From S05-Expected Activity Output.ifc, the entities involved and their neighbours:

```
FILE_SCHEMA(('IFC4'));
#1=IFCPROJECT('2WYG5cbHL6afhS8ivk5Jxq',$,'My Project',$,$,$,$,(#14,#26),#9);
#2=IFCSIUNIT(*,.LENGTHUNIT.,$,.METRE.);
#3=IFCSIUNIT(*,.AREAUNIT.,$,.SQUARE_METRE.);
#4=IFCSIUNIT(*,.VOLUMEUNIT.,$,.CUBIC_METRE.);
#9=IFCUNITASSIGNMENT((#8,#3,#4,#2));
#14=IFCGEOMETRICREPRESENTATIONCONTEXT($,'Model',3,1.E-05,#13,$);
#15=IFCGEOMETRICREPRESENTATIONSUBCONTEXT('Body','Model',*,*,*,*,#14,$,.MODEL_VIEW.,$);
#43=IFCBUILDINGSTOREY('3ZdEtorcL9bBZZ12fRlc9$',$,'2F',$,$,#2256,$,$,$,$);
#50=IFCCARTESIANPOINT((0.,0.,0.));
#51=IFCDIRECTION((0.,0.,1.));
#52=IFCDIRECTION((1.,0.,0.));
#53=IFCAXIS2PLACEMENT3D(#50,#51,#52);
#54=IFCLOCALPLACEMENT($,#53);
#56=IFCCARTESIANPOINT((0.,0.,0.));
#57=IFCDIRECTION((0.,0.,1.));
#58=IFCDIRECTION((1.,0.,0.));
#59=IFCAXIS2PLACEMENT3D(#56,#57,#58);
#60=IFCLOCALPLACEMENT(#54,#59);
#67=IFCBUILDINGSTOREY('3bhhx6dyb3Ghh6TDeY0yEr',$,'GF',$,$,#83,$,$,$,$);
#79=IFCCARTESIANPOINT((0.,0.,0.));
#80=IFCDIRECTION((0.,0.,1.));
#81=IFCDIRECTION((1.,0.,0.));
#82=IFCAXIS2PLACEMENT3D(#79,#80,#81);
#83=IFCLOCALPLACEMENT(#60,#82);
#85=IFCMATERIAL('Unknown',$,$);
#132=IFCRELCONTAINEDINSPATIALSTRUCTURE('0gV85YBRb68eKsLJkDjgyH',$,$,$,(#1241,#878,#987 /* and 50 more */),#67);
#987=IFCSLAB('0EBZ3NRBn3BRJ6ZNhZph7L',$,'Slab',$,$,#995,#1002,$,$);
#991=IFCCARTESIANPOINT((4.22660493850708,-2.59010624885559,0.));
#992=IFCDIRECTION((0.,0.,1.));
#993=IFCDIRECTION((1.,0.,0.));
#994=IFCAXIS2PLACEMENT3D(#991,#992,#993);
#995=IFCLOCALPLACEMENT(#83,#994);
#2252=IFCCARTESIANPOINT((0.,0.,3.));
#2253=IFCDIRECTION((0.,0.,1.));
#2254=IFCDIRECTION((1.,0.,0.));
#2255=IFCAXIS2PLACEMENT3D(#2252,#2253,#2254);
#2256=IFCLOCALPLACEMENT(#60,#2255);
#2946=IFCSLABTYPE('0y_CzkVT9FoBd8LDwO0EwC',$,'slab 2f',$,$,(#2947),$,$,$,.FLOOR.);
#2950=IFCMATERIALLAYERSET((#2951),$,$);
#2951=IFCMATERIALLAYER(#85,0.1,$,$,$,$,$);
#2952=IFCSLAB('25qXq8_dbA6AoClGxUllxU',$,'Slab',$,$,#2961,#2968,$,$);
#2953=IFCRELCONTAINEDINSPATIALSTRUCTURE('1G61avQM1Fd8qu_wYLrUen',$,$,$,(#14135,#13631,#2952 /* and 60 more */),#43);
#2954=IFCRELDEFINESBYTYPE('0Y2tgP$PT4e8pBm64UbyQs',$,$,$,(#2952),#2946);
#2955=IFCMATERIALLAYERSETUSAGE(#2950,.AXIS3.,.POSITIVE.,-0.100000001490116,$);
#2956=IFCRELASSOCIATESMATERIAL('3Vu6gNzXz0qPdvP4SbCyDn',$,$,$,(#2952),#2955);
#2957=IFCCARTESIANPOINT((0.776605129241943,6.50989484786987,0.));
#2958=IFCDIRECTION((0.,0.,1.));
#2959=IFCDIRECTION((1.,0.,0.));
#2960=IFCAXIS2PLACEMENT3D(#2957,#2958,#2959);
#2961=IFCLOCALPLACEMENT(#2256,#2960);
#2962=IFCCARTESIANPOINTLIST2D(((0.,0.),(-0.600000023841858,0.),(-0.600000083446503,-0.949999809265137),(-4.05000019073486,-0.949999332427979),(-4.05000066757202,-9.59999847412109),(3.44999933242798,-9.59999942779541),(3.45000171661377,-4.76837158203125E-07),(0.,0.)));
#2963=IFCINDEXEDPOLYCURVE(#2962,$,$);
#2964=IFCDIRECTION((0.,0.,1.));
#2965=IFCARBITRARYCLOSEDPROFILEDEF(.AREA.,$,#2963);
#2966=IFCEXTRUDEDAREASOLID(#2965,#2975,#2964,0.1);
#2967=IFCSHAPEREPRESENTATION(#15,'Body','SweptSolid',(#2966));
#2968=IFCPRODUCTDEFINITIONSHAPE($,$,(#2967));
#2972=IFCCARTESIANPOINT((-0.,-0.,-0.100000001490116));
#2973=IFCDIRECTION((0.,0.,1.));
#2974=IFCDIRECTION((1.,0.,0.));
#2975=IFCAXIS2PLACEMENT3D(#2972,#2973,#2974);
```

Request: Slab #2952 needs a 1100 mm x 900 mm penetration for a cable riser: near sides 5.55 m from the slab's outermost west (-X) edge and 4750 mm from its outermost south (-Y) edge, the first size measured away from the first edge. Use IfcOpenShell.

```python
import numpy as np
import ifcopenshell
import ifcopenshell.api.feature
import ifcopenshell.api.geometry
import ifcopenshell.api.root
import ifcopenshell.geom
import ifcopenshell.util.placement
import ifcopenshell.util.representation
import ifcopenshell.util.shape
import ifcopenshell.util.unit

model = ifcopenshell.open("S05-Expected Activity Output.ifc")
unit_scale = ifcopenshell.util.unit.calculate_unit_scale(model)
settings = ifcopenshell.geom.settings()


def volume(element):
    """Net volume in cubic metres, openings subtracted."""
    shape = ifcopenshell.geom.create_shape(settings, element)
    return ifcopenshell.util.shape.get_volume(shape.geometry)


slab = model.by_guid("25qXq8_dbA6AoClGxUllxU")
before = volume(slab)

# Extent in the slab's own axes, in metres. The edges named are its -X and -Y sides.
slab_shape = ifcopenshell.geom.create_shape(settings, slab)
vertices = ifcopenshell.util.shape.get_vertices(slab_shape.geometry)
x_min, y_min, bottom = vertices.min(axis=0)
top = vertices[:, 2].max()

opening = ifcopenshell.api.root.create_entity(model, ifc_class="IfcOpeningElement", name="Cable riser opening", predefined_type="OPENING")
context = ifcopenshell.util.representation.get_context(model, "Model", "Body", "MODEL_VIEW")
width, depth = 1.1, 0.9
outline = [(0.0, 0.0), (width, 0.0), (width, depth), (0.0, depth), (0.0, 0.0)]
# Overshoot both faces by 50 mm so the cut is clean.
shape = ifcopenshell.api.geometry.add_slab_representation(
    model, context=context, depth=top - bottom + 0.1, polyline=outline
)
ifcopenshell.api.geometry.assign_representation(model, product=opening, representation=shape)

matrix = ifcopenshell.util.placement.get_local_placement(slab.ObjectPlacement)
matrix[:, 3] = matrix @ np.append(np.array([x_min + 5.55, y_min + 4.75, bottom - 0.05]) / unit_scale, 1.0)
ifcopenshell.api.geometry.edit_object_placement(model, product=opening, matrix=matrix, is_si=False)
ifcopenshell.api.feature.add_feature(model, feature=opening, element=slab)

after = volume(slab)

print(f"slab volume {before:.3f} -> {after:.3f} m3")

model.write("S05-Expected Activity Output_v2.ifc")
```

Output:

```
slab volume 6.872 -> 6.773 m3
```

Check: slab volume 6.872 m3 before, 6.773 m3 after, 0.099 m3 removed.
